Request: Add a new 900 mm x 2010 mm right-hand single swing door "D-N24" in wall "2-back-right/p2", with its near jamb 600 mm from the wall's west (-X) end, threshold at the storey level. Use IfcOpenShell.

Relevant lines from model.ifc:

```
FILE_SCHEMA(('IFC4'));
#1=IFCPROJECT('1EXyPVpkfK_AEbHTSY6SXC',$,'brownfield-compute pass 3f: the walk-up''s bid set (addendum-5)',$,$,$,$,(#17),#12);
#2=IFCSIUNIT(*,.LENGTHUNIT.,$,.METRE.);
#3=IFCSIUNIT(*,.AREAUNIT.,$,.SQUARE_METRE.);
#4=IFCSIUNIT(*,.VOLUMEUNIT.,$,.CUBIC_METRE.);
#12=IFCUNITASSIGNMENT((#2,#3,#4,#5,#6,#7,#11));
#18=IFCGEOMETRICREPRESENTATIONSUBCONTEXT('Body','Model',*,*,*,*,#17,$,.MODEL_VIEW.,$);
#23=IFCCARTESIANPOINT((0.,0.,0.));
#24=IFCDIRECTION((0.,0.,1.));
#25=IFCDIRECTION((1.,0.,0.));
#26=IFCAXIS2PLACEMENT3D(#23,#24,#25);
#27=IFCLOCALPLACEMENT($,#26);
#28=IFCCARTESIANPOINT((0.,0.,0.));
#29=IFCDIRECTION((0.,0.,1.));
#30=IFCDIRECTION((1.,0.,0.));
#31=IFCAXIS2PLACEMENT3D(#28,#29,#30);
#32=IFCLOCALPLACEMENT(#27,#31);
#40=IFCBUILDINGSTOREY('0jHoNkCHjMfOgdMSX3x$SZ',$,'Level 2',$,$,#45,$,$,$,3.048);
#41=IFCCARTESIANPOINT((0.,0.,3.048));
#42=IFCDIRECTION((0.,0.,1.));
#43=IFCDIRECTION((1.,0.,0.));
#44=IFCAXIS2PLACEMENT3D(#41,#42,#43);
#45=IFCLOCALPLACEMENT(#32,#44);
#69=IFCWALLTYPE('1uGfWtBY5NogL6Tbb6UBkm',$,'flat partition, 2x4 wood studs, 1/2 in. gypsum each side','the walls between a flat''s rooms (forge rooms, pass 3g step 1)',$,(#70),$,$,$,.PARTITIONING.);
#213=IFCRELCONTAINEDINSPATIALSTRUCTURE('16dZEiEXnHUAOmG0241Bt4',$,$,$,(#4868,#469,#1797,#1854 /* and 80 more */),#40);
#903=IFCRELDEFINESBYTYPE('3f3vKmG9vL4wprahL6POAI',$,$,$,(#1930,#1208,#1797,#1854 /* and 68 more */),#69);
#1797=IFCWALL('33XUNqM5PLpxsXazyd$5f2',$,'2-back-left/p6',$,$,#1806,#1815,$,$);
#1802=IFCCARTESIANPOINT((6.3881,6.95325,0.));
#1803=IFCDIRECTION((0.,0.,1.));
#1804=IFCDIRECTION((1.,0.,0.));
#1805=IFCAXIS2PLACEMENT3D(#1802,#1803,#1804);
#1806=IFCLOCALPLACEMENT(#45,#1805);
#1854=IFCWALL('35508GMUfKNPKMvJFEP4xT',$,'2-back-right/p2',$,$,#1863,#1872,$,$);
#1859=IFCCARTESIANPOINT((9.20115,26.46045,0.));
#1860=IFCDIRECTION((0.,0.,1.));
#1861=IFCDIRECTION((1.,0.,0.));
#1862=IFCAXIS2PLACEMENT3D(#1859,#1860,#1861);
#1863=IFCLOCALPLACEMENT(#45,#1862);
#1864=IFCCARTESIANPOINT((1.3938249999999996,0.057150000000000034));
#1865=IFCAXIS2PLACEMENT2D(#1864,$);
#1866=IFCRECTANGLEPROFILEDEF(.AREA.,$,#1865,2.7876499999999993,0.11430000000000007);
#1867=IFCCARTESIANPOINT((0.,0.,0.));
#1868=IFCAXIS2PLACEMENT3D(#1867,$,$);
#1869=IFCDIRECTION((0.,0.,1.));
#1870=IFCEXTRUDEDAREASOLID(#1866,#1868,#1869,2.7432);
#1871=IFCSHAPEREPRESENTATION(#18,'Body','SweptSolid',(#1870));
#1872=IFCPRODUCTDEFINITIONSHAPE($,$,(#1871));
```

```python
import numpy as np
import ifcopenshell
import ifcopenshell.api.feature
import ifcopenshell.api.geometry
import ifcopenshell.api.root
import ifcopenshell.api.spatial
import ifcopenshell.geom
import ifcopenshell.util.element
import ifcopenshell.util.placement
import ifcopenshell.util.representation
import ifcopenshell.util.shape
import ifcopenshell.util.unit

model = ifcopenshell.open("model.ifc")
unit_scale = ifcopenshell.util.unit.calculate_unit_scale(model)
settings = ifcopenshell.geom.settings()


def volume(element):
    """Net volume in cubic metres, openings subtracted."""
    shape = ifcopenshell.geom.create_shape(settings, element)
    return ifcopenshell.util.shape.get_volume(shape.geometry)


wall = model.by_guid("35508GMUfKNPKMvJFEP4xT")
storey = ifcopenshell.util.element.get_container(wall, ifc_class="IfcBuildingStorey")
context = ifcopenshell.util.representation.get_context(model, "Model", "Body", "MODEL_VIEW")
before = volume(wall)

width, height, from_end, sill = 0.9, 2.01, 0.6, 0.0  # metres

# The wall runs along its own X axis, and the end named is its -X end.
wall_shape = ifcopenshell.geom.create_shape(settings, wall)
x, y, z = ifcopenshell.util.shape.get_vertices(wall_shape.geometry).T
start = x.min() + from_end
face, thickness = float(y.min()), float(y.max() - y.min())
wall_matrix = ifcopenshell.util.placement.get_local_placement(wall.ObjectPlacement)
level = ifcopenshell.util.placement.get_local_placement(storey.ObjectPlacement)[2, 3]


def in_wall(x, y):
    """Placement at x, y metres in the wall's axes, at sill height."""
    matrix = wall_matrix.copy()
    matrix[:, 3] = wall_matrix @ np.array([x / unit_scale, y / unit_scale, 0.0, 1.0])
    matrix[2, 3] = level + sill / unit_scale
    return matrix


# Opening: a box that overshoots both wall faces by 50 mm.
opening = ifcopenshell.api.root.create_entity(model, ifc_class="IfcOpeningElement", predefined_type="OPENING")
box = ifcopenshell.api.geometry.add_wall_representation(
    model, context=context, length=width, height=height, thickness=thickness + 0.1
)
ifcopenshell.api.geometry.assign_representation(model, product=opening, representation=box)
ifcopenshell.api.geometry.edit_object_placement(model, product=opening, matrix=in_wall(start, face - 0.05), is_si=False)
ifcopenshell.api.feature.add_feature(model, feature=opening, element=wall)

door = ifcopenshell.api.root.create_entity(model, ifc_class="IfcDoor", name="D-N24", predefined_type="DOOR")
door.OverallWidth, door.OverallHeight = width / unit_scale, height / unit_scale
door.OperationType = "SINGLE_SWING_RIGHT"
body = ifcopenshell.api.geometry.add_door_representation(
    model,
    context=context,
    overall_width=door.OverallWidth,
    overall_height=door.OverallHeight,
    operation_type="SINGLE_SWING_RIGHT",
    lining_properties={"LiningDepth": thickness / unit_scale, "ThresholdDepth": thickness / unit_scale},
)
ifcopenshell.api.geometry.assign_representation(model, product=door, representation=body)
ifcopenshell.api.spatial.assign_container(model, products=[door], relating_structure=storey)
ifcopenshell.api.feature.add_filling(model, opening=opening, element=door)

# The lining spans the wall, so the door starts at the wall face.
ifcopenshell.api.geometry.edit_object_placement(model, product=door, matrix=in_wall(start, face), is_si=False)

after = volume(wall)

print(f"wall volume {before:.3f} -> {after:.3f} m3")

model.write("model_edited.ifc")
```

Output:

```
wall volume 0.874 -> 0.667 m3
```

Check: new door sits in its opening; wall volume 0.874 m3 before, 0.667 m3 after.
